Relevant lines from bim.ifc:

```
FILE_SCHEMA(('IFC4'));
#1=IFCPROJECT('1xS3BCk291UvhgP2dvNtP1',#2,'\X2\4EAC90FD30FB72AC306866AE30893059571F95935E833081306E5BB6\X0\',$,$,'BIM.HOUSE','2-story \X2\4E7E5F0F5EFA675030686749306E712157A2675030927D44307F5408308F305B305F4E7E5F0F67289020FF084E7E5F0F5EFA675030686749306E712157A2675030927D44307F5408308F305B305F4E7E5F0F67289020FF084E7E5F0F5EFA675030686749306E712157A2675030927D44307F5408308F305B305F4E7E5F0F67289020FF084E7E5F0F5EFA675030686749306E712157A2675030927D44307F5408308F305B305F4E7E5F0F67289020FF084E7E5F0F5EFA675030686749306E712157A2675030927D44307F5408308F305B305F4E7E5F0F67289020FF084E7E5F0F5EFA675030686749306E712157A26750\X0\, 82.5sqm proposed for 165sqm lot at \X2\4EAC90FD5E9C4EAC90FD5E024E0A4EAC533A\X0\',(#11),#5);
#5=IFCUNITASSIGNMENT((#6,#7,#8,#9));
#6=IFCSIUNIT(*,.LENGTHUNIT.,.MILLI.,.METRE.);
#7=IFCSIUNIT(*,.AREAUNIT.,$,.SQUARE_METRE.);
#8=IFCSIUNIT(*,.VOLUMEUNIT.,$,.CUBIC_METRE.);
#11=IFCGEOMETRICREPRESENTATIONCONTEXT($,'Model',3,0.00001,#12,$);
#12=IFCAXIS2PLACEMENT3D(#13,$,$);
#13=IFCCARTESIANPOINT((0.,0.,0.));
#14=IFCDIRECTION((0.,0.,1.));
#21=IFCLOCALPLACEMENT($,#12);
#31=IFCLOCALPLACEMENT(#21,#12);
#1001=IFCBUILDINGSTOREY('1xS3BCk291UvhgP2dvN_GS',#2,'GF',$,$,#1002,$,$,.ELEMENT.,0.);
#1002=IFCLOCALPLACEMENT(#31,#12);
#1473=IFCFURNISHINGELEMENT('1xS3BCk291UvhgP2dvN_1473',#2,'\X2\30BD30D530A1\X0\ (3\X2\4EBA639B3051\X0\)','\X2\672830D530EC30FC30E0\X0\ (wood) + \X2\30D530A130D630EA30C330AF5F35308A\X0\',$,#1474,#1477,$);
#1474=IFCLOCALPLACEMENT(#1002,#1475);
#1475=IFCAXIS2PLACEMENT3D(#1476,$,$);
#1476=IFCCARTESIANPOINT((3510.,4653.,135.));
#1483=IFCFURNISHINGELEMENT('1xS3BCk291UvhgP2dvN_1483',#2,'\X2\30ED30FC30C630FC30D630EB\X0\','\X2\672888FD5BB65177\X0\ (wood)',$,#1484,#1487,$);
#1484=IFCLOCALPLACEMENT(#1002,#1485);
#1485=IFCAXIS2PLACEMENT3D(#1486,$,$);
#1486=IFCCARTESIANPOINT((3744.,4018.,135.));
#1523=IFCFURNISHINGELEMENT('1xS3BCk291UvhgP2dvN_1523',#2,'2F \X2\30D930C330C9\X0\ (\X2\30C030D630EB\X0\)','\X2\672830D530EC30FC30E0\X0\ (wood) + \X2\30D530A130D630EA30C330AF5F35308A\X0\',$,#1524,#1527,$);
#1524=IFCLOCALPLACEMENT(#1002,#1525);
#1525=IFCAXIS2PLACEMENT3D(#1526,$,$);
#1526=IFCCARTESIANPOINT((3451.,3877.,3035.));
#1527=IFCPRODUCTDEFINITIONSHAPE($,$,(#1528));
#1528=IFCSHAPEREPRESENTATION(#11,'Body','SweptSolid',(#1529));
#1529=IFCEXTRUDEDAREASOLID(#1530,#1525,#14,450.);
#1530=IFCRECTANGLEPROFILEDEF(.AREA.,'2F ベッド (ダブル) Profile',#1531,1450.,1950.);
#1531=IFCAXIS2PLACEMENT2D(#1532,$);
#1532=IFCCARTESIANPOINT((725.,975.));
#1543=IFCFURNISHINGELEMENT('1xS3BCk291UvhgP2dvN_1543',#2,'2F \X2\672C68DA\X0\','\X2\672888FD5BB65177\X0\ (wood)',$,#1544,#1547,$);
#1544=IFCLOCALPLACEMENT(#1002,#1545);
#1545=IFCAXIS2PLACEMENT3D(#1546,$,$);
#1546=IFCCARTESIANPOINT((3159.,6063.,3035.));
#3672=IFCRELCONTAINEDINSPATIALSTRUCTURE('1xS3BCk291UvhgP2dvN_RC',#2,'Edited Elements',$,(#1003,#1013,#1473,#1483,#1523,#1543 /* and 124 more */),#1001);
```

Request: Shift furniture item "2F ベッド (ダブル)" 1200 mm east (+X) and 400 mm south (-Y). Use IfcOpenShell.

```python
import ifcopenshell
import ifcopenshell.api.geometry
import ifcopenshell.util.placement
import ifcopenshell.util.unit

model = ifcopenshell.open("bim.ifc")
unit_scale = ifcopenshell.util.unit.calculate_unit_scale(model)

item = model.by_id(1523)
matrix = ifcopenshell.util.placement.get_local_placement(item.ObjectPlacement)
matrix[0, 3] += 1.2 / unit_scale
matrix[1, 3] -= 0.4 / unit_scale
ifcopenshell.api.geometry.edit_object_placement(model, product=item, matrix=matrix, is_si=False)

print(ifcopenshell.util.placement.get_local_placement(item.ObjectPlacement).round(3) + 0.0)

model.write("bim_edited.ifc")
```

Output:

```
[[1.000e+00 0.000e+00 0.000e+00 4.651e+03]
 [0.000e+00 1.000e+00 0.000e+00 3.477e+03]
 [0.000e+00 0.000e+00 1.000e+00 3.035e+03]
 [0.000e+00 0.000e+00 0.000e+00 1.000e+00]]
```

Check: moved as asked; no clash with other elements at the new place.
